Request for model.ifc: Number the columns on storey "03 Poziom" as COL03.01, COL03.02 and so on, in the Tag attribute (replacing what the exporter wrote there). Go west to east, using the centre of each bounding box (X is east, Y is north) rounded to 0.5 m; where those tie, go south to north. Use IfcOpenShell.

First a look at what the model holds.

```python
import ifcopenshell
import ifcopenshell.util.element
import ifcopenshell.util.placement

model = ifcopenshell.open("model.ifc")
print(model.schema)
storey = next(s for s in model.by_type("IfcBuildingStorey") if s.Name == "03 Poziom")
columns = [e for e in ifcopenshell.util.element.get_decomposition(storey) if e.is_a("IfcColumn")]
for e in sorted(columns, key=lambda e: e.id()):
    origin = ifcopenshell.util.placement.get_local_placement(e.ObjectPlacement)[:3, 3]
    print(e.id(), e.Tag, e.Name, origin.round(2) + 0.0, sep=" | ")
```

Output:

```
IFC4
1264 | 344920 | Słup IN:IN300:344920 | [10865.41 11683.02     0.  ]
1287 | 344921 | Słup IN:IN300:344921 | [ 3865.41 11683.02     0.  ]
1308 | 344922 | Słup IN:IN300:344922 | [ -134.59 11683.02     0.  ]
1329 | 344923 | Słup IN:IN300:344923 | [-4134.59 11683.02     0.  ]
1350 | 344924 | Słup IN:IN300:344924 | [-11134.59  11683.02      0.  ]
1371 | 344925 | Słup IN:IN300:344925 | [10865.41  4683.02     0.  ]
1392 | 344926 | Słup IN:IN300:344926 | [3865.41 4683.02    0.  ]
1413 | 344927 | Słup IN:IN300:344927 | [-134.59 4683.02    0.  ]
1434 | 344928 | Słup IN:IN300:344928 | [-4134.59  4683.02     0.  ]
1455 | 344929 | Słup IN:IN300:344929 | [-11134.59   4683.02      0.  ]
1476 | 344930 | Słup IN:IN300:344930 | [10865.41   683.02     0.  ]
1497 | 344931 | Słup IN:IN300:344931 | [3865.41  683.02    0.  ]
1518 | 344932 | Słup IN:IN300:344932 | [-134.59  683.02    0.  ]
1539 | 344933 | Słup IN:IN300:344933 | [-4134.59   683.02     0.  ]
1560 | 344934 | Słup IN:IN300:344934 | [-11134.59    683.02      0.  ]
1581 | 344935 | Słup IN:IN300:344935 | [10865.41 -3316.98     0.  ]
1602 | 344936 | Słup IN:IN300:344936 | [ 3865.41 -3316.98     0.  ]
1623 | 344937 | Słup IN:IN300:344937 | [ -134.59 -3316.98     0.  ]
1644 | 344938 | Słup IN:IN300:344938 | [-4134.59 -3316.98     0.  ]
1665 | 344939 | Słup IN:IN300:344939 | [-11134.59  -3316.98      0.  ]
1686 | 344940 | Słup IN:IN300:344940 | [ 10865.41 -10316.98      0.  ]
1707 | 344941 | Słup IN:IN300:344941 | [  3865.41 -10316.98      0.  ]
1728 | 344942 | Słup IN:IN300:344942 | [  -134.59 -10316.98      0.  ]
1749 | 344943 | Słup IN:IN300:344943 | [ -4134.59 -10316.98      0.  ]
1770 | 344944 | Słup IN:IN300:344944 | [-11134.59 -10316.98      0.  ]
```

```python
import ifcopenshell
import ifcopenshell.geom
import ifcopenshell.util.element
import ifcopenshell.util.shape

model = ifcopenshell.open("model.ifc")
settings = ifcopenshell.geom.settings()
settings.set("use-world-coords", True)


def centre(element):
    shape = ifcopenshell.geom.create_shape(settings, element)
    return ifcopenshell.util.shape.get_bbox_centroid(shape.geometry)


storey = next(s for s in model.by_type("IfcBuildingStorey") if s.Name == "03 Poziom")
columns = [e for e in ifcopenshell.util.element.get_decomposition(storey) if e.is_a("IfcColumn")]

# Insertion points can sit at a corner or the storey origin, so sort by the geometry (in metres).
centres = {e: centre(e) for e in columns}
columns.sort(key=lambda e: (round(centres[e][0] / 0.5), centres[e][1]))

for i, e in enumerate(columns, start=1):
    number = f"COL03.{i:02d}"
    e.Tag = number
    print(e.id(), number)

model.write("model_rev.ifc")
```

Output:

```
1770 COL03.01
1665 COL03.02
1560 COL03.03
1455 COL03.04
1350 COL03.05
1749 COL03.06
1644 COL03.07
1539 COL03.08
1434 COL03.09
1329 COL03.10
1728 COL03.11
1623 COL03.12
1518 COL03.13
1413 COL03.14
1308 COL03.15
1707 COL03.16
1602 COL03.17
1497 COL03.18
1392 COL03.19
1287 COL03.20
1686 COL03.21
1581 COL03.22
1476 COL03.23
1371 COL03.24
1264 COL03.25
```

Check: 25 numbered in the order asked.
